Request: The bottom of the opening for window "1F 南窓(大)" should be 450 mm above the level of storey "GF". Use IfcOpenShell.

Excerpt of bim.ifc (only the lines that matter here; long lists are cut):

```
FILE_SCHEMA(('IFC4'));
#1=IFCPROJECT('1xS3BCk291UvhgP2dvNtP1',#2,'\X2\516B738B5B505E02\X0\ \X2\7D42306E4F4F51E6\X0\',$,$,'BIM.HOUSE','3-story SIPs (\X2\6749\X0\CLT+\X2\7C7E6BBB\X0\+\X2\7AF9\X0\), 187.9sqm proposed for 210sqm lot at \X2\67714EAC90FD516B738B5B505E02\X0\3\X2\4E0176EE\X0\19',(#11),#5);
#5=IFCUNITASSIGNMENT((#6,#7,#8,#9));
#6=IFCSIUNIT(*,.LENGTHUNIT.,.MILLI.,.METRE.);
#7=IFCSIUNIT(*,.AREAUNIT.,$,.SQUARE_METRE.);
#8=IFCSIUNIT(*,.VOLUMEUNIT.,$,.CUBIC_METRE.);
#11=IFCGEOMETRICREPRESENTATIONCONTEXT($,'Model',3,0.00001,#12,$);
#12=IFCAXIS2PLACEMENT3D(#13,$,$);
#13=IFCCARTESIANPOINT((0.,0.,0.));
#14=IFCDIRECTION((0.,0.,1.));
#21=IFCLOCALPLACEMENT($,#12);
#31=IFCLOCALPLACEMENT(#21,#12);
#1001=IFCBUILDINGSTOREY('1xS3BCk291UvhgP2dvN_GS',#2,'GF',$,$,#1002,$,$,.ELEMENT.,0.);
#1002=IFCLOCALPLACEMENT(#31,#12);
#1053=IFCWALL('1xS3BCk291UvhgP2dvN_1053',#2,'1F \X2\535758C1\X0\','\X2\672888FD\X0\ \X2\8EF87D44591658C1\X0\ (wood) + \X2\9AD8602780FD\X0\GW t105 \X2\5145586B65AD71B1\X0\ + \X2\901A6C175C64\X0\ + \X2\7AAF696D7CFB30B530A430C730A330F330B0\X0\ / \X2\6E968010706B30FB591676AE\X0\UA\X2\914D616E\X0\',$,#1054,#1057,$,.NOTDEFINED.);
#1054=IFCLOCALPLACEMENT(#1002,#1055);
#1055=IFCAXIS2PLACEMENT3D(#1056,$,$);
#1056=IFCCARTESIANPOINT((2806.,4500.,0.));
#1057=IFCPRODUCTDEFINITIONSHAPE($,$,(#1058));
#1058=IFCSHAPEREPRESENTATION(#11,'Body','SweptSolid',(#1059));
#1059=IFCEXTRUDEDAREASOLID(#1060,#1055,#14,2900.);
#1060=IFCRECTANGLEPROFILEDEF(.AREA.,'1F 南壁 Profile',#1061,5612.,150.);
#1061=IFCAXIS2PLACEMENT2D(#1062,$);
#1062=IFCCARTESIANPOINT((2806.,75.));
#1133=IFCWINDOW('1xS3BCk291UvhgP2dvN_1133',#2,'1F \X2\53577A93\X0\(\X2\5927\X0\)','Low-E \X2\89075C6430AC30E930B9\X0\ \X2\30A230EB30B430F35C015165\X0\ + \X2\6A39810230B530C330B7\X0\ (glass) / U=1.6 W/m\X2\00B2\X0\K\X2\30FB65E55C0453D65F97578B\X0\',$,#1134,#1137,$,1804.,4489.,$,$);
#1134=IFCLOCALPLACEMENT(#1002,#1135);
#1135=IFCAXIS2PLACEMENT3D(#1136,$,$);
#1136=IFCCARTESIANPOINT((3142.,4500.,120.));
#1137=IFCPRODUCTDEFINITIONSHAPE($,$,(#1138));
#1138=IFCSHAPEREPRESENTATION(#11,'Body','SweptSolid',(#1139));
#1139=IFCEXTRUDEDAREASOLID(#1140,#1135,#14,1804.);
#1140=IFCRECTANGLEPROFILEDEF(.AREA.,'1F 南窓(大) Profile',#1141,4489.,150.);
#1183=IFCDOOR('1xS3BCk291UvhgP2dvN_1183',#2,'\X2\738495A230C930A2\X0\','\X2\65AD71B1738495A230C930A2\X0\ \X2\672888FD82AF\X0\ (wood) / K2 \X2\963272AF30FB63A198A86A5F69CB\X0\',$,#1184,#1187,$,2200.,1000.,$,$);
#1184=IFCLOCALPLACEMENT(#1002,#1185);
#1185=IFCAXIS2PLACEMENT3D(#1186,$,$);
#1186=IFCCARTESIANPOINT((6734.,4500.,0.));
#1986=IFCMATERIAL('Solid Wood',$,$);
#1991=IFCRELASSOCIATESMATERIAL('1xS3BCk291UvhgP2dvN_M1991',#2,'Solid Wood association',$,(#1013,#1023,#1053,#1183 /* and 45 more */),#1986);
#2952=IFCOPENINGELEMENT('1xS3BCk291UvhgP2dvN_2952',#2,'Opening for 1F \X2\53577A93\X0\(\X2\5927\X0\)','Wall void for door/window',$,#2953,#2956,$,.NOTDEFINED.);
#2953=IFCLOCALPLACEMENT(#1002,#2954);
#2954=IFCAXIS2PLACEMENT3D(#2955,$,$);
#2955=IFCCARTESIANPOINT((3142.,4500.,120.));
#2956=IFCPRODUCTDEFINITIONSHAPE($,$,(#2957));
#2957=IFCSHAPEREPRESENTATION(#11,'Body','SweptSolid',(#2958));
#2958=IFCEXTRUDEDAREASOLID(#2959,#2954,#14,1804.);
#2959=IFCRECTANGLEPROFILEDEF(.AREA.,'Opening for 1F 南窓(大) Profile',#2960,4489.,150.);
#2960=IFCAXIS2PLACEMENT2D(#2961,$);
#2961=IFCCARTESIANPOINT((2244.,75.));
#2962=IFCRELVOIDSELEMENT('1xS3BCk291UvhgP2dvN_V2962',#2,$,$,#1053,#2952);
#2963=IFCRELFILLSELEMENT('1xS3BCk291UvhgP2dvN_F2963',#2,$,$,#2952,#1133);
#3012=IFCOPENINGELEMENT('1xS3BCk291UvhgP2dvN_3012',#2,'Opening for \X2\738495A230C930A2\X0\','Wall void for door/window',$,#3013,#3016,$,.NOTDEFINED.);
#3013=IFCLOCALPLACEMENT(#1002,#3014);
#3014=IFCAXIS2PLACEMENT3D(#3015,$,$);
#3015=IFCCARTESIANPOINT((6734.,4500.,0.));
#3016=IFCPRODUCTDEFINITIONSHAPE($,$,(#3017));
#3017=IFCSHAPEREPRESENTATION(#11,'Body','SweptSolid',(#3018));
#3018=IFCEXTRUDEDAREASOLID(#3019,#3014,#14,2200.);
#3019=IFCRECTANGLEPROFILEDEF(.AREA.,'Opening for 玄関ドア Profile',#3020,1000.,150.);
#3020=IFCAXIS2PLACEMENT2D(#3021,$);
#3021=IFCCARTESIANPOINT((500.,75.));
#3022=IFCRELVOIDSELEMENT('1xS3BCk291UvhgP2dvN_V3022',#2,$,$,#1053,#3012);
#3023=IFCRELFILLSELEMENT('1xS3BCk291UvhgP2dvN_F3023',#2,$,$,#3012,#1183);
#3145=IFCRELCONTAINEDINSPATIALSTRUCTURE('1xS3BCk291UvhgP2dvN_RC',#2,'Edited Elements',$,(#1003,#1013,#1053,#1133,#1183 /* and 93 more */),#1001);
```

```python
import numpy as np
import ifcopenshell
import ifcopenshell.api.geometry
import ifcopenshell.geom
import ifcopenshell.util.element
import ifcopenshell.util.placement
import ifcopenshell.util.shape
import ifcopenshell.util.unit

model = ifcopenshell.open("bim.ifc")
unit_scale = ifcopenshell.util.unit.calculate_unit_scale(model)

window = model.by_id(1133)
opening = window.FillsVoids[0].RelatingOpeningElement
storey = ifcopenshell.util.element.get_container(window, ifc_class="IfcBuildingStorey")
level = ifcopenshell.util.placement.get_local_placement(storey.ObjectPlacement)[2, 3]

# The opening's origin need not be at the sill, so measure its lowest point.
shape = ifcopenshell.geom.create_shape(ifcopenshell.geom.settings(), opening)
bottom = ifcopenshell.util.shape.get_shape_bottom_elevation(shape, shape.geometry) / unit_scale
dz = level + 450.0 - bottom

shift = np.array([0.0, 0.0, dz])
# The window is not placed relative to its opening, so move both.
for product in (opening, window):
    matrix = ifcopenshell.util.placement.get_local_placement(product.ObjectPlacement)
    matrix[:3, 3] += shift
    ifcopenshell.api.geometry.edit_object_placement(model, product=product, matrix=matrix, is_si=False)

print(f"moved by {dz * unit_scale:+.3f} m")

model.write("bim_rev.ifc")
```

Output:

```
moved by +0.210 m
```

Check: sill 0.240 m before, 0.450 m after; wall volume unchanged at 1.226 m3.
